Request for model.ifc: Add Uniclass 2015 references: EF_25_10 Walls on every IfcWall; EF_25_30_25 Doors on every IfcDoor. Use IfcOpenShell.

First a look at what the model holds.

```python
import ifcopenshell

model = ifcopenshell.open("model.ifc")
print(model.schema)
print("classifications:", [c.Name for c in model.by_type("IfcClassification")])
for ifc_class in ("IfcDoor", "IfcRoof", "IfcStair", "IfcWall", "IfcWindow"):
    print(ifc_class, len(model.by_type(ifc_class)))
```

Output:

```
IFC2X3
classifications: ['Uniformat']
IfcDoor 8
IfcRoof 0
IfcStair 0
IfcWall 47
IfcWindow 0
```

```python
import ifcopenshell
import ifcopenshell.api.classification

model = ifcopenshell.open("model.ifc")

# IFC2X3 requires Source and Edition and has no link from the project to the system.
system = model.create_entity("IfcClassification", Source="NBS", Edition="2015", Name="Uniclass 2015")

codes = {
    "IfcWall": ("EF_25_10", "Walls"),
    "IfcDoor": ("EF_25_30_25", "Doors"),
}
for ifc_class, (code, name) in codes.items():
    products = model.by_type(ifc_class)
    ifcopenshell.api.classification.add_reference(
        model, products=products, classification=system, identification=code, name=name
    )
    print(code, len(products))

model.write("model_rev.ifc")
```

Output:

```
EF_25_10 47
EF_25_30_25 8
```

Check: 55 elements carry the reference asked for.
